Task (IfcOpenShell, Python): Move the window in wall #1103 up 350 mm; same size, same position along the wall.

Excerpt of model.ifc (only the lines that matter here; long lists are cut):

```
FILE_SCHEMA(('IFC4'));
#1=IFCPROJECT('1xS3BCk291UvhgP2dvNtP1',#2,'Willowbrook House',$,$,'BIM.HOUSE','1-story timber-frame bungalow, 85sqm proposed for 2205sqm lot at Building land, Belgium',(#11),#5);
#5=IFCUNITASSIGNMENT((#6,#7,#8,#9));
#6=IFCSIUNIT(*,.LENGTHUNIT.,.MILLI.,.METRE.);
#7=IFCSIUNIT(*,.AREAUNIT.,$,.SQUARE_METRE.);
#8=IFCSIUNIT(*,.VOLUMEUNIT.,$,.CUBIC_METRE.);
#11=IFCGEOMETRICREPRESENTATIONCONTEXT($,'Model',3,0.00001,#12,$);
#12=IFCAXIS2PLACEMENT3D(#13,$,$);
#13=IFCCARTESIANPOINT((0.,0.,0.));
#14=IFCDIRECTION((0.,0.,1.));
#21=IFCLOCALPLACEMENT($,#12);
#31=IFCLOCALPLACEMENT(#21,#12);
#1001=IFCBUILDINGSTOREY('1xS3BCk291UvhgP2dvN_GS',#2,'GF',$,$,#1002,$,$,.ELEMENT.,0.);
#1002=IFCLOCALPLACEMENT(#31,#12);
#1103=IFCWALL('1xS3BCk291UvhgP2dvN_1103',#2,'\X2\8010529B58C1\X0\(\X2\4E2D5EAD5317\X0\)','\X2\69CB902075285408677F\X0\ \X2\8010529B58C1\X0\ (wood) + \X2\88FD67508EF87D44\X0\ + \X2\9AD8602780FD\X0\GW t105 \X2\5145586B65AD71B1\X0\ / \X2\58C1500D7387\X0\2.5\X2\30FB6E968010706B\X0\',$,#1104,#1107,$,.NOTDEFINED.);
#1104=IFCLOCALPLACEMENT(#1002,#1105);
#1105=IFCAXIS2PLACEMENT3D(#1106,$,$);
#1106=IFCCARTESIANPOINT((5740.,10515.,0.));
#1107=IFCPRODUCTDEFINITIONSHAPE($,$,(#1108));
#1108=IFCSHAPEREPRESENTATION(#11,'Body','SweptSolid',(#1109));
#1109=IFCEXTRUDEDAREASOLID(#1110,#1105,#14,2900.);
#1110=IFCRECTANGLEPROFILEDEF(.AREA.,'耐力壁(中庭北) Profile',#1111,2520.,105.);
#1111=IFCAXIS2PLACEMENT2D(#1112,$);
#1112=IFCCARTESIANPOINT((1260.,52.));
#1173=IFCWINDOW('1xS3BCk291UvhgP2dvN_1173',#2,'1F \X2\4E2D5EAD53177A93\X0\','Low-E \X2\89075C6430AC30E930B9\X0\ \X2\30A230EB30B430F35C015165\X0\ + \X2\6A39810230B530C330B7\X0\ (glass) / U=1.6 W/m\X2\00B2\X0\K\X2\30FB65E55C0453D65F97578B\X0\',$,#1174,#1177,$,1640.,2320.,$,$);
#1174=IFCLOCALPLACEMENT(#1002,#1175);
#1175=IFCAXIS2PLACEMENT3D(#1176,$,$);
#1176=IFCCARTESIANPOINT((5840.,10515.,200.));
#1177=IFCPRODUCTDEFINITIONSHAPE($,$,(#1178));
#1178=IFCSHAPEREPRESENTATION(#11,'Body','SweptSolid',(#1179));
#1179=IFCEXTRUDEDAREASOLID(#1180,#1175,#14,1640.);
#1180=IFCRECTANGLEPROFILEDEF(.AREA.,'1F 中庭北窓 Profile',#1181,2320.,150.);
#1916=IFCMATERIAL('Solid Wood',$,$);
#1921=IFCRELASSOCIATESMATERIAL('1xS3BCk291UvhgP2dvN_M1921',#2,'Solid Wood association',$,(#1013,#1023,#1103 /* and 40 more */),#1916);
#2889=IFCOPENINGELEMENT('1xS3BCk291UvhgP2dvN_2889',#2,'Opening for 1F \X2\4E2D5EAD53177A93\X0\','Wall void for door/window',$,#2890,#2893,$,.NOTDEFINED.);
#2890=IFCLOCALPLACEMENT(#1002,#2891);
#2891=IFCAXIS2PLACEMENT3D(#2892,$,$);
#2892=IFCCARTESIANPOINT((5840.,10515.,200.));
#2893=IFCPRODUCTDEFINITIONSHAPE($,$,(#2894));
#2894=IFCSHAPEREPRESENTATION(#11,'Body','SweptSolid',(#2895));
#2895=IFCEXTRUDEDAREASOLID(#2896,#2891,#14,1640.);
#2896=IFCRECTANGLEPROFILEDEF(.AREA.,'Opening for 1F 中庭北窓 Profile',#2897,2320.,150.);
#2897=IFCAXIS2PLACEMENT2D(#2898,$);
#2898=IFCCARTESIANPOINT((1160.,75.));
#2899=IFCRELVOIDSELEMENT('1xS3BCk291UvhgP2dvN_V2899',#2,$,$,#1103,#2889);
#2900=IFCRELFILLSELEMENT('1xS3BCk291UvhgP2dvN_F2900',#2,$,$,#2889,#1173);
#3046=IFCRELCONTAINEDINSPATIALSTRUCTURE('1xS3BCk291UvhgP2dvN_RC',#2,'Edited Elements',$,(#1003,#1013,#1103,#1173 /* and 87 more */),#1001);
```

```python
import numpy as np
import ifcopenshell
import ifcopenshell.api.geometry
import ifcopenshell.util.placement
import ifcopenshell.util.unit

model = ifcopenshell.open("model.ifc")
unit_scale = ifcopenshell.util.unit.calculate_unit_scale(model)

window = model.by_id(1173)
opening = window.FillsVoids[0].RelatingOpeningElement
dz = 350.0

shift = np.array([0.0, 0.0, dz])
# The window is not placed relative to its opening, so move both.
for product in (opening, window):
    matrix = ifcopenshell.util.placement.get_local_placement(product.ObjectPlacement)
    matrix[:3, 3] += shift
    ifcopenshell.api.geometry.edit_object_placement(model, product=product, matrix=matrix, is_si=False)

print(f"moved by {dz * unit_scale:+.3f} m")

model.write("model_rev.ifc")
```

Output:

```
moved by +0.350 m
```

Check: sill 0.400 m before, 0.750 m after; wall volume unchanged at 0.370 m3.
